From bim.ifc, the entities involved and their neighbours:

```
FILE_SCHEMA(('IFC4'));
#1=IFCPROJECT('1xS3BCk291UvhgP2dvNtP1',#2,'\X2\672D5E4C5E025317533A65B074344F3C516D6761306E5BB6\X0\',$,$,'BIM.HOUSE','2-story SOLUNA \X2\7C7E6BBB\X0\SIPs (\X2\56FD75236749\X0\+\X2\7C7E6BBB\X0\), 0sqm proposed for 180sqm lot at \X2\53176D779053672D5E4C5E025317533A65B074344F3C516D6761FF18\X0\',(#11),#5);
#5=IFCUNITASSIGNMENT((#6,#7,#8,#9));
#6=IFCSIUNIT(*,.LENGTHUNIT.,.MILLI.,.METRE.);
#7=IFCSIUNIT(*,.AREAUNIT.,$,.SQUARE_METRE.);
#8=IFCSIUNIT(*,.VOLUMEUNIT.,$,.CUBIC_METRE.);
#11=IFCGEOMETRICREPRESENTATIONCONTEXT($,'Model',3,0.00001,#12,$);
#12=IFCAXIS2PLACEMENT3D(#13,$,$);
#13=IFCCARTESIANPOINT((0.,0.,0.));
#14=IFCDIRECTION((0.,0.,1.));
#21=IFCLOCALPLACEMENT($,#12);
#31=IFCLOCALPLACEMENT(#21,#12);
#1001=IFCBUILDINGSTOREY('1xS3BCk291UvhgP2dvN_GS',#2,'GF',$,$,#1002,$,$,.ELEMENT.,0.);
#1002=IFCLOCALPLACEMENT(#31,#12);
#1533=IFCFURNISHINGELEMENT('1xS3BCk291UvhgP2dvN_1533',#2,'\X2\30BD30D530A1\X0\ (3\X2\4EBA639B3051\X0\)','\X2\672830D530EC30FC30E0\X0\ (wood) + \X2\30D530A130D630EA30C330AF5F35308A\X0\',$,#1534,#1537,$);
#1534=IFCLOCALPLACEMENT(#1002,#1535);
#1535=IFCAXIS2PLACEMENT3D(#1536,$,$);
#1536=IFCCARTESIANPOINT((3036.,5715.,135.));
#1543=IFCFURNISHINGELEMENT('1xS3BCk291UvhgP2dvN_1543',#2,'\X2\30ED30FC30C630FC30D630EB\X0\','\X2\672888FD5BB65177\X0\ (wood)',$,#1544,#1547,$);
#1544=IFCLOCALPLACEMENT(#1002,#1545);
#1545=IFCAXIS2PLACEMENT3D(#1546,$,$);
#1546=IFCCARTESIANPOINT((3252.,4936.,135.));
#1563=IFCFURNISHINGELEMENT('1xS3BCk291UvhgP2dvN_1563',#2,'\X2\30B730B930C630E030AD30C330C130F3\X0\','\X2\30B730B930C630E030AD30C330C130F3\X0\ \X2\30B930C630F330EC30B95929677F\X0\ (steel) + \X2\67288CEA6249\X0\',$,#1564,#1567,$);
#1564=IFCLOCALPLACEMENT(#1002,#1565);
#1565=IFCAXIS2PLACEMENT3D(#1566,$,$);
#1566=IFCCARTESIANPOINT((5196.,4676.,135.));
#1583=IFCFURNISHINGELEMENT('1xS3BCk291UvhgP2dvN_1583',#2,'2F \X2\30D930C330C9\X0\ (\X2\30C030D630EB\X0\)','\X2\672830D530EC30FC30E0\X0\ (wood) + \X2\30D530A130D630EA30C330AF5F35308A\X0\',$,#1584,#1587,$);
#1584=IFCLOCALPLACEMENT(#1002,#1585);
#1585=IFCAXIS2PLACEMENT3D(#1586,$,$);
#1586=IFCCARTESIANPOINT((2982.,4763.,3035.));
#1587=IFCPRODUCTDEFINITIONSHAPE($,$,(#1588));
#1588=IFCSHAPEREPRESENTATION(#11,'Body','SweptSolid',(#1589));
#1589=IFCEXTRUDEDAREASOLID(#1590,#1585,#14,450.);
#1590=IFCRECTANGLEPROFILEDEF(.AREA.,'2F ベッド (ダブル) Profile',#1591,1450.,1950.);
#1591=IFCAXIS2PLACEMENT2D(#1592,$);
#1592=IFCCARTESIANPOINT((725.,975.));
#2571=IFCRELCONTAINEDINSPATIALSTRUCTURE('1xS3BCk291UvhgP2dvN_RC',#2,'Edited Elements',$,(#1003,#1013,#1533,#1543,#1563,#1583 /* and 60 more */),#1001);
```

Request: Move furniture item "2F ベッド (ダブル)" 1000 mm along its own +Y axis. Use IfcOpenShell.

```python
import ifcopenshell
import ifcopenshell.api.geometry
import ifcopenshell.util.placement
import ifcopenshell.util.unit

model = ifcopenshell.open("bim.ifc")
unit_scale = ifcopenshell.util.unit.calculate_unit_scale(model)

item = model.by_id(1583)
matrix = ifcopenshell.util.placement.get_local_placement(item.ObjectPlacement)
matrix[:3, 3] += matrix[:3, 1] * 1 / unit_scale
ifcopenshell.api.geometry.edit_object_placement(model, product=item, matrix=matrix, is_si=False)

print(ifcopenshell.util.placement.get_local_placement(item.ObjectPlacement).round(3) + 0.0)

model.write("bim_updated.ifc")
```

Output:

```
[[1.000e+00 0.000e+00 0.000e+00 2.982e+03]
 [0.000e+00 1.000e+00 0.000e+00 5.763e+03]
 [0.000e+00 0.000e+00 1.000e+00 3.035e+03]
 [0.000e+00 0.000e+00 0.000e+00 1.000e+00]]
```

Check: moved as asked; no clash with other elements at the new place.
